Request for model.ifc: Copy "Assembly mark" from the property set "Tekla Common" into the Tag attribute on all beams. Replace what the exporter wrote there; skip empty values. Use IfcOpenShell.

First a look at what the model holds.

```python
import ifcopenshell
import ifcopenshell.util.element

model = ifcopenshell.open("model.ifc")
print(model.schema)
beams = model.by_type("IfcBeam")
print(len(beams), "beams")
for e in beams[:8]:
    source = ifcopenshell.util.element.get_pset(e, "Tekla Common", "Assembly mark")
    target = e.Tag
    print(e.id(), repr(source), repr(target), sep=" | ")
```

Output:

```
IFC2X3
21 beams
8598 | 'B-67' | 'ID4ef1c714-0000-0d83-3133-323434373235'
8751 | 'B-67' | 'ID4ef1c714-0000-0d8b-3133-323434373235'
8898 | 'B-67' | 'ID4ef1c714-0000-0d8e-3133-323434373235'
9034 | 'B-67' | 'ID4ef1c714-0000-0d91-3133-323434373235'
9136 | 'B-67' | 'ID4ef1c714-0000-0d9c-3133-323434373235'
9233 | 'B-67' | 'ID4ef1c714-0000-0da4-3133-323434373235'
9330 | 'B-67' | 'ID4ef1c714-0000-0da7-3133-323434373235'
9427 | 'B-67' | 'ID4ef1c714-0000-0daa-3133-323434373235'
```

```python
import ifcopenshell
import ifcopenshell.util.element

model = ifcopenshell.open("model.ifc")

count = 0
for e in model.by_type("IfcBeam"):
    value = ifcopenshell.util.element.get_pset(e, "Tekla Common", "Assembly mark")
    current = e.Tag
    if not value or not value.strip() or current == value:
        continue
    e.Tag = value
    count += 1

print(count, "beams updated")

model.write("model_v2.ifc")
```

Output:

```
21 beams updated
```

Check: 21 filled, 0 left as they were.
